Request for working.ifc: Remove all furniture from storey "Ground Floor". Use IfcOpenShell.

First a look at what the model holds.

```python
import ifcopenshell
import ifcopenshell.util.element

model = ifcopenshell.open("working.ifc")
print(model.schema)
storey = next(s for s in model.by_type("IfcBuildingStorey") if s.Name == "Ground Floor")
furniture = [e for e in ifcopenshell.util.element.get_decomposition(storey) if e.is_a("IfcFurnishingElement")]
seen = {}
for e in furniture:
    element_type = ifcopenshell.util.element.get_type(e)
    name = element_type.Name if element_type not in (None, e) else None
    seen[name] = seen.get(name, 0) + 1
for name, count in sorted(seen.items(), key=str):
    print(count, "x", name)
```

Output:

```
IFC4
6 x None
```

```python
import ifcopenshell
import ifcopenshell.api.root
import ifcopenshell.util.element

model = ifcopenshell.open("working.ifc")

storey = next(s for s in model.by_type("IfcBuildingStorey") if s.Name == "Ground Floor")
furniture = [e for e in ifcopenshell.util.element.get_decomposition(storey) if e.is_a("IfcFurnishingElement")]

for e in furniture:
    ifcopenshell.api.root.remove_product(model, product=e)
print(len(furniture), "removed")

model.write("working_updated.ifc")
```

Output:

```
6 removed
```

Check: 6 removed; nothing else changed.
